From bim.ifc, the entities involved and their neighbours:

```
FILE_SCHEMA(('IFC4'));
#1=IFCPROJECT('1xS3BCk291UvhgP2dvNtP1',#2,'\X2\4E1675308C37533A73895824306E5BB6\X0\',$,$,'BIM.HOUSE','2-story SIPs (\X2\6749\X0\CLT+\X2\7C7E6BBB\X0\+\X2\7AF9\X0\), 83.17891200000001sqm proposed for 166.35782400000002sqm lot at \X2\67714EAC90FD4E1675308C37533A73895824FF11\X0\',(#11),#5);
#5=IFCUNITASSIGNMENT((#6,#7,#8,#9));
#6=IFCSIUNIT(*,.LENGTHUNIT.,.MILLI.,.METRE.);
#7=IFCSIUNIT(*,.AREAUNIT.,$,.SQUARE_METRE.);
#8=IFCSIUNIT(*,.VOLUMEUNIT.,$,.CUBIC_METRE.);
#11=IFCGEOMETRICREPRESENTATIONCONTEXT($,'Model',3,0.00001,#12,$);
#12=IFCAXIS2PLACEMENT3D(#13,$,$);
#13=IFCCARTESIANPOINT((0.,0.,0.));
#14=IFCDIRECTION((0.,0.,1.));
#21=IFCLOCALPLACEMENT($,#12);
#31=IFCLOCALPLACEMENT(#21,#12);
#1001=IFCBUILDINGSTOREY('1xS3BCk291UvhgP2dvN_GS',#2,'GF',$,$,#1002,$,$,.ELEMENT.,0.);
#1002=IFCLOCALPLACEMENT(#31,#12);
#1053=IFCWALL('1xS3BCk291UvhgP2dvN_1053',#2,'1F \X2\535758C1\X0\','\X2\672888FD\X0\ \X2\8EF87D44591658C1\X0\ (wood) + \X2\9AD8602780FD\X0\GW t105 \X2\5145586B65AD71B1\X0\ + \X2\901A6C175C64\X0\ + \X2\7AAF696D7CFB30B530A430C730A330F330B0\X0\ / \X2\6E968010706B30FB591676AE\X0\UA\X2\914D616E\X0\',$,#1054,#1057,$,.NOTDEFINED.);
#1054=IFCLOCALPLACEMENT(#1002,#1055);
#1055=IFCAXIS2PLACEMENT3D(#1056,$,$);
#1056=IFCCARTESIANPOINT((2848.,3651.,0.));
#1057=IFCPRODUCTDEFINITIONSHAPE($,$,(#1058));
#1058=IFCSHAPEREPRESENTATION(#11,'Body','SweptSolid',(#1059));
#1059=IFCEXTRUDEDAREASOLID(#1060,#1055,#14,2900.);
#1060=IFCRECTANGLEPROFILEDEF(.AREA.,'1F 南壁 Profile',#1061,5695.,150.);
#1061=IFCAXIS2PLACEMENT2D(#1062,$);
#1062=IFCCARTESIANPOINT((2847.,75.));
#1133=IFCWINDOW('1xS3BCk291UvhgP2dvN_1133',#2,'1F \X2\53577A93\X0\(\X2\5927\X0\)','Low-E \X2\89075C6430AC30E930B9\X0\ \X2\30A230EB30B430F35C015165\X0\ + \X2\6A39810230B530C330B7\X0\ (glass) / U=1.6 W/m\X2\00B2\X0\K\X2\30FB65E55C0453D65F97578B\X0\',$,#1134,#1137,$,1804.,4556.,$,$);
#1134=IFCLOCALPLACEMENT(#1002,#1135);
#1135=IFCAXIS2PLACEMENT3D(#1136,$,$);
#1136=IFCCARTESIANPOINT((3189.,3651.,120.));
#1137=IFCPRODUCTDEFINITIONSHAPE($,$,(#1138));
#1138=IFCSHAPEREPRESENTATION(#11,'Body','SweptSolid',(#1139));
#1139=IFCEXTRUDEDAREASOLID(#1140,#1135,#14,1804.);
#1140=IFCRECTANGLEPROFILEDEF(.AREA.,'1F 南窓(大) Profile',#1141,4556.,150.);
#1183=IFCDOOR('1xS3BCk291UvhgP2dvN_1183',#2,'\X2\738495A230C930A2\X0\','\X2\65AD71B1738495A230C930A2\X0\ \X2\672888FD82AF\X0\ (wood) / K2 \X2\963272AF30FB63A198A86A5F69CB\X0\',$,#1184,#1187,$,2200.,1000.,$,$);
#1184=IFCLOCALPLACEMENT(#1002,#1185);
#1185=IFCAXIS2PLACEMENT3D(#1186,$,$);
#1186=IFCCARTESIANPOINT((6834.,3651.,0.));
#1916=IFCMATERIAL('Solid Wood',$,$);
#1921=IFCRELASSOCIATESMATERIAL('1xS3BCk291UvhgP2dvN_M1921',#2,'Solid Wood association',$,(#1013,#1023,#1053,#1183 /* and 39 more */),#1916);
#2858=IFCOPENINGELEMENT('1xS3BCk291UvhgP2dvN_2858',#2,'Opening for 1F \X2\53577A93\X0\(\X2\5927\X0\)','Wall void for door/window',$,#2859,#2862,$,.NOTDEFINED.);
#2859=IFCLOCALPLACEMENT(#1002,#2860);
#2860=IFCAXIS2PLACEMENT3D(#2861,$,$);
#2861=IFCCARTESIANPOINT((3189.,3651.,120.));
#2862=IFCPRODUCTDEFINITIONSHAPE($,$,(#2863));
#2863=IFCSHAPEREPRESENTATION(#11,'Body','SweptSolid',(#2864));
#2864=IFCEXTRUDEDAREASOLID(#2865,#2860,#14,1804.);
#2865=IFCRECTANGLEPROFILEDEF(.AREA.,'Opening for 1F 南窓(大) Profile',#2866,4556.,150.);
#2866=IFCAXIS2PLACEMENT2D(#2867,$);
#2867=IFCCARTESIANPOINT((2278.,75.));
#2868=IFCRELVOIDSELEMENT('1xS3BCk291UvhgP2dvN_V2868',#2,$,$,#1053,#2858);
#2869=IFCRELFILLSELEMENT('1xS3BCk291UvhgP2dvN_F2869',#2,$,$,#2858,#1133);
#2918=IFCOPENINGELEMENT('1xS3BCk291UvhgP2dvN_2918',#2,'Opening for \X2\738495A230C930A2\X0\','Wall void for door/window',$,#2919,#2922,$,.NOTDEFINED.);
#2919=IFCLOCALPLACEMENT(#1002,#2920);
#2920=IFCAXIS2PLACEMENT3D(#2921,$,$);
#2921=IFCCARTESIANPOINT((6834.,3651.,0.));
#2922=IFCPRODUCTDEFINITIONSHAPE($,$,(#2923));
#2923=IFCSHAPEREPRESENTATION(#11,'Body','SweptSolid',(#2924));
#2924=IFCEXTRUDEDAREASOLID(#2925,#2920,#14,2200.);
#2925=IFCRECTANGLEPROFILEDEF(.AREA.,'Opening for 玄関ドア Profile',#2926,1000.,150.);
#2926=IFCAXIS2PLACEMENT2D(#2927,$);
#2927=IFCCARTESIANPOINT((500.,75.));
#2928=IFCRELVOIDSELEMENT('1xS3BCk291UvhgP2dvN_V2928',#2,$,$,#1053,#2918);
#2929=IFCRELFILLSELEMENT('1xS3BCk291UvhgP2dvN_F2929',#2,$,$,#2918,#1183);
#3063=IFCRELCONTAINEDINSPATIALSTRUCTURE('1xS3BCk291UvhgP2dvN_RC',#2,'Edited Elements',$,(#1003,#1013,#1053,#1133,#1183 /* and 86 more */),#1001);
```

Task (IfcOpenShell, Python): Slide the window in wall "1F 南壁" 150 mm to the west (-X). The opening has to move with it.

```python
import ifcopenshell
import ifcopenshell.api.geometry
import ifcopenshell.util.placement
import ifcopenshell.util.unit

model = ifcopenshell.open("bim.ifc")
unit_scale = ifcopenshell.util.unit.calculate_unit_scale(model)

window = model.by_guid("1xS3BCk291UvhgP2dvN_1133")
opening = window.FillsVoids[0].RelatingOpeningElement
wall = opening.VoidsElements[0].RelatingBuildingElement

wall_matrix = ifcopenshell.util.placement.get_local_placement(wall.ObjectPlacement)
shift = wall_matrix[:3, 0] * -0.15 / unit_scale
before = ifcopenshell.util.placement.get_local_placement(window.ObjectPlacement)[:3, 3].copy()

# The window is not placed relative to its opening, so move both.
for product in (opening, window):
    matrix = ifcopenshell.util.placement.get_local_placement(product.ObjectPlacement)
    matrix[:3, 3] += shift
    ifcopenshell.api.geometry.edit_object_placement(model, product=product, matrix=matrix, is_si=False)

after = ifcopenshell.util.placement.get_local_placement(window.ObjectPlacement)[:3, 3]
print("window moved by", (after - before).round(3) + 0.0)

model.write("bim_edited.ifc")
```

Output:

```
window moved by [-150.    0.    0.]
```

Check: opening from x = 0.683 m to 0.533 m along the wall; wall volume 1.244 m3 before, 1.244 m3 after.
